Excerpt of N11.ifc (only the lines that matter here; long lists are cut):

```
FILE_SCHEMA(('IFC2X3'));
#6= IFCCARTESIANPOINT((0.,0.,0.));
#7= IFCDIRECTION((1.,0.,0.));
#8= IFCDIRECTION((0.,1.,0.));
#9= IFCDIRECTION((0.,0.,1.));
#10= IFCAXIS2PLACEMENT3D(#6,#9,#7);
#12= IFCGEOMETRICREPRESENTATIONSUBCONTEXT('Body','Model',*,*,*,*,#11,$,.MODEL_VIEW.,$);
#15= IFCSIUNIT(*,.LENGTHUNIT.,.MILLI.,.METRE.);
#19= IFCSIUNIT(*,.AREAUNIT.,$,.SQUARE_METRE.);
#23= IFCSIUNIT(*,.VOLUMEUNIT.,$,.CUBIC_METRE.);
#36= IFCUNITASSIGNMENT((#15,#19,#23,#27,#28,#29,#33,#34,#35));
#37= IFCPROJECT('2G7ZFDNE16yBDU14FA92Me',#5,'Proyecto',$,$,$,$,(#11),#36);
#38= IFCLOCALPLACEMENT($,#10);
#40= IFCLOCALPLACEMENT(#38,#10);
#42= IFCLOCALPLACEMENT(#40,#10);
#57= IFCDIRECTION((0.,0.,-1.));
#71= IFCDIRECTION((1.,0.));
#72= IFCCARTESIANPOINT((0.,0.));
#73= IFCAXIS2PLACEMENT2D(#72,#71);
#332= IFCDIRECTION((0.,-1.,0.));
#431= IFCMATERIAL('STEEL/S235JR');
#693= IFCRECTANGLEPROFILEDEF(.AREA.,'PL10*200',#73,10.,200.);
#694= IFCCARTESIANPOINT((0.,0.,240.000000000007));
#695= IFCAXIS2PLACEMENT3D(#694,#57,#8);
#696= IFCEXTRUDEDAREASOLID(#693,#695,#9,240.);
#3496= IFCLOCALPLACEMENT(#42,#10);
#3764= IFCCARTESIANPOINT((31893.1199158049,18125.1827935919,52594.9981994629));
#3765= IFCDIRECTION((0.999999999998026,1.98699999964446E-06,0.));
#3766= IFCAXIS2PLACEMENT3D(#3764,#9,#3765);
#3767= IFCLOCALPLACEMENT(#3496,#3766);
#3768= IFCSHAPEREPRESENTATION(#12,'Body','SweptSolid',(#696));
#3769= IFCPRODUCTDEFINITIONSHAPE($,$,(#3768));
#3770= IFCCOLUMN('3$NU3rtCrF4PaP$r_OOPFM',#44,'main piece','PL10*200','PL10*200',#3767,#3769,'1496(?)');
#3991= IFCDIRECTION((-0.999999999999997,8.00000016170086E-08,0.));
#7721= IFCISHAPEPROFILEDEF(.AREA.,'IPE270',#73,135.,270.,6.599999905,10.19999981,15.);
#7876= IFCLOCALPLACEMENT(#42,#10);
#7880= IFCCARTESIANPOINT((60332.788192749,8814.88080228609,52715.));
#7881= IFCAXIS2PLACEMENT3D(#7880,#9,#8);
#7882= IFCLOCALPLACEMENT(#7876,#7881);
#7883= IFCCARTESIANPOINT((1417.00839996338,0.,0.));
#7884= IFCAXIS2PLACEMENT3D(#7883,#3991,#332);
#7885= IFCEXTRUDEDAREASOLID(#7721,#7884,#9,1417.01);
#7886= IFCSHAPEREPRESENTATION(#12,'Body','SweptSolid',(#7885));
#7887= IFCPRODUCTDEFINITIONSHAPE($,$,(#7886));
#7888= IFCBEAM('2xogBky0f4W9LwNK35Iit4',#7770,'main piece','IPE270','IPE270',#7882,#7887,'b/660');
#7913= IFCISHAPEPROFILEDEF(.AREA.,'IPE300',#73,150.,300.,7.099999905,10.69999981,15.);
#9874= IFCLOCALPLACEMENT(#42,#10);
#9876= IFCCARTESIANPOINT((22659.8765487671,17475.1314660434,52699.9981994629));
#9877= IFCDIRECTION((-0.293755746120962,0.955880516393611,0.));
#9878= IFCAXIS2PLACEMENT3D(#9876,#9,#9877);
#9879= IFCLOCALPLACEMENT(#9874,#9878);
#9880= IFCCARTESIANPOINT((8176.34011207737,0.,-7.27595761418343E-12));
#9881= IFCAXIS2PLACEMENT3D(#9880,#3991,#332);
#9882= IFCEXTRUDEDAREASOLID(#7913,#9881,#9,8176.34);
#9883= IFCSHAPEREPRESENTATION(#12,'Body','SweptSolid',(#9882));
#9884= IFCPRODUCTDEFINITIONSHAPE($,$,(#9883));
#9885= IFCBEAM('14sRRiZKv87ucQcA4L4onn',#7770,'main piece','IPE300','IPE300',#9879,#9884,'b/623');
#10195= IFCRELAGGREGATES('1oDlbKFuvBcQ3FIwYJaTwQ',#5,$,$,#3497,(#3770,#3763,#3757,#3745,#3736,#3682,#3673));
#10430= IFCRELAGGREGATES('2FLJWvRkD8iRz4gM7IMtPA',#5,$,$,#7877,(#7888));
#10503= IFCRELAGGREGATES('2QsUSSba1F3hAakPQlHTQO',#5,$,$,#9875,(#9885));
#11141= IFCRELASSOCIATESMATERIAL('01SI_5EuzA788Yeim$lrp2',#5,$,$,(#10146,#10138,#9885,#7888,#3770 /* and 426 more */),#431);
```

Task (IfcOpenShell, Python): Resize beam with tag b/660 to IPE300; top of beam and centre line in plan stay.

```python
import ifcopenshell
import ifcopenshell.util.element
import ifcopenshell.util.representation

model = ifcopenshell.open("N11.ifc")

member = model.by_guid("2xogBky0f4W9LwNK35Iit4")
source = next(p for p in model.by_type("IfcIShapeProfileDef") if p.ProfileName == "IPE300")

body = ifcopenshell.util.representation.get_representation(member, "Model", "Body")
solid = body.Items[0]
old_profile = solid.SweptArea

# Copy the section's sizes but keep this member's own profile position.
profile = ifcopenshell.util.element.copy(model, source)
# Profiles are centred, so shift by half the change in depth to hold the top.
shift = (old_profile.OverallDepth - profile.OverallDepth) / 2
x, y = old_profile.Position.Location.Coordinates
up = (0.0, 1.0)  # upwards, in the solid's own plane
location = model.createIfcCartesianPoint((x + up[0] * shift, y + up[1] * shift))
profile.Position = model.createIfcAxis2Placement2D(location, old_profile.Position.RefDirection)
solid.SweptArea = profile
if not model.get_total_inverses(old_profile):
    ifcopenshell.util.element.remove_deep2(model, old_profile)
member.Description = member.Description.replace("IPE270", "IPE300")
member.ObjectType = member.ObjectType.replace("IPE270", "IPE300")

print(solid.SweptArea)

model.write("N11-out.ifc")
```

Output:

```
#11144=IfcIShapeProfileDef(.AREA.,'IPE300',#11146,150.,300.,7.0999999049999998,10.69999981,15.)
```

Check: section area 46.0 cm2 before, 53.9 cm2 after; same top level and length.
